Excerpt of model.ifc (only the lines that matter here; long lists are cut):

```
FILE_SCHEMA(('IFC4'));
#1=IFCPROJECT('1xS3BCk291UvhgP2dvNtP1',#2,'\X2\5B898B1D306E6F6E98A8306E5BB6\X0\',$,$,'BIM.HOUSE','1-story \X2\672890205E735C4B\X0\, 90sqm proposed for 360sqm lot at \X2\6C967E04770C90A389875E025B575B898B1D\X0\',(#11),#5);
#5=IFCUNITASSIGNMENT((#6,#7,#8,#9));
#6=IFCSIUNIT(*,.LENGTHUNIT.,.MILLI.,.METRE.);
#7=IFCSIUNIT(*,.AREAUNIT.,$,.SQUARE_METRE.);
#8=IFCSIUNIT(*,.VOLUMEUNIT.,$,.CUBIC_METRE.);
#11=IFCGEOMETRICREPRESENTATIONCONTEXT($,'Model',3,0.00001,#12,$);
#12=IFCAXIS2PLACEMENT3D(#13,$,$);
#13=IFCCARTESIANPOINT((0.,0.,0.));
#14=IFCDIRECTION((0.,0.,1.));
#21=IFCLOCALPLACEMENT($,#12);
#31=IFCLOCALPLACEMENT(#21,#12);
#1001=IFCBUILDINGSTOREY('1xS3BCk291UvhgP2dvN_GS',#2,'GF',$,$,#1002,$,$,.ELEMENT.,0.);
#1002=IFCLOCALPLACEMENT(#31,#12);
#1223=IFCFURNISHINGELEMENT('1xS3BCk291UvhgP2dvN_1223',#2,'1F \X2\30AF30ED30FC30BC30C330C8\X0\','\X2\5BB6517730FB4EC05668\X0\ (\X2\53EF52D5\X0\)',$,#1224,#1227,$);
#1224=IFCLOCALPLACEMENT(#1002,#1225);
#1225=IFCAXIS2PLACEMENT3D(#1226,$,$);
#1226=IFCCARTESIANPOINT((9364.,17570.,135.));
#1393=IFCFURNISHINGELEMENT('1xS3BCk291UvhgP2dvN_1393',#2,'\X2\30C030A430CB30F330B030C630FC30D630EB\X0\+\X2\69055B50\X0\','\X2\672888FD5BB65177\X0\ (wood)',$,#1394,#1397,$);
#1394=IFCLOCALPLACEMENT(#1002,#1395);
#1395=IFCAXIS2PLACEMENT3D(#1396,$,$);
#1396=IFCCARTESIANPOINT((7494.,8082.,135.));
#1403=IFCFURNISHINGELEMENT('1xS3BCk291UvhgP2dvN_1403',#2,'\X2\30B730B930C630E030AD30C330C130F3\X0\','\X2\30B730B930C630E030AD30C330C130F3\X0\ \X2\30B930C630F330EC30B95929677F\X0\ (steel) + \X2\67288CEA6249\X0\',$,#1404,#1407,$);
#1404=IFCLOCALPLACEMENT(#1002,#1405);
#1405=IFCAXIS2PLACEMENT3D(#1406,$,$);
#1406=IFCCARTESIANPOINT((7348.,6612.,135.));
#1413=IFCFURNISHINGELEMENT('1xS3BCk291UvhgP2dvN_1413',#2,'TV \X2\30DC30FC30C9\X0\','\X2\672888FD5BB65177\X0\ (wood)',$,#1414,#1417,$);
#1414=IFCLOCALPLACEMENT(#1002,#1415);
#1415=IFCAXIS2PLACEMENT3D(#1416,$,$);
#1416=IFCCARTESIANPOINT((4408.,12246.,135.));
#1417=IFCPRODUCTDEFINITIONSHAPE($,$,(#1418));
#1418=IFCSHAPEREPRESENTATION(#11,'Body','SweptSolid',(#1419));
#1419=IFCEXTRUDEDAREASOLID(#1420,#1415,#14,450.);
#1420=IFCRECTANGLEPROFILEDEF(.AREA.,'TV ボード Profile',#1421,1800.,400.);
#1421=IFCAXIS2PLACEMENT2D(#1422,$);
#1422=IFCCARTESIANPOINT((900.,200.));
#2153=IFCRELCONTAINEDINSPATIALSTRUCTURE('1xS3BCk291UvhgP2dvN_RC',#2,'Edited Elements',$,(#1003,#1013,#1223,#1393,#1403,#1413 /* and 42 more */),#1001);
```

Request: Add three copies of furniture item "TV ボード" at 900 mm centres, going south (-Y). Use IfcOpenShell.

```python
import numpy as np
import ifcopenshell
import ifcopenshell.api.geometry
import ifcopenshell.api.root
import ifcopenshell.util.element
import ifcopenshell.util.placement

model = ifcopenshell.open("model.ifc")


def reuse_history(source, copy):
    """copy_class also copies each property set's owner history, people and application; keep the originals."""
    for rel in copy.IsDefinedBy:
        if rel.is_a("IfcRelDefinesByProperties") and (history := rel.RelatingPropertyDefinition.OwnerHistory):
            rel.RelatingPropertyDefinition.OwnerHistory = source.OwnerHistory
            ifcopenshell.util.element.remove_deep2(model, history)


source = model.by_guid("1xS3BCk291UvhgP2dvN_1413")
base = ifcopenshell.util.placement.get_local_placement(source.ObjectPlacement)
step = np.array([0.0, -1.0, 0.0]) * 900.0

for i in range(1, 4):
    copy = ifcopenshell.api.root.copy_class(model, product=source)
    copy.Representation = ifcopenshell.util.element.copy_deep(
        model, source.Representation, exclude=["IfcGeometricRepresentationContext", "IfcRepresentationMap"]
    )
    reuse_history(source, copy)
    matrix = base.copy()
    matrix[:3, 3] += i * step
    print("added at", matrix[:3, 3].round(3) + 0.0)
    ifcopenshell.api.geometry.edit_object_placement(model, product=copy, matrix=matrix, is_si=False)

model.write("model_rev.ifc")
```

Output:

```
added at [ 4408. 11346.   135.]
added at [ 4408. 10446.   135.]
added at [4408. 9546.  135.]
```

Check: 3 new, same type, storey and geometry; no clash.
